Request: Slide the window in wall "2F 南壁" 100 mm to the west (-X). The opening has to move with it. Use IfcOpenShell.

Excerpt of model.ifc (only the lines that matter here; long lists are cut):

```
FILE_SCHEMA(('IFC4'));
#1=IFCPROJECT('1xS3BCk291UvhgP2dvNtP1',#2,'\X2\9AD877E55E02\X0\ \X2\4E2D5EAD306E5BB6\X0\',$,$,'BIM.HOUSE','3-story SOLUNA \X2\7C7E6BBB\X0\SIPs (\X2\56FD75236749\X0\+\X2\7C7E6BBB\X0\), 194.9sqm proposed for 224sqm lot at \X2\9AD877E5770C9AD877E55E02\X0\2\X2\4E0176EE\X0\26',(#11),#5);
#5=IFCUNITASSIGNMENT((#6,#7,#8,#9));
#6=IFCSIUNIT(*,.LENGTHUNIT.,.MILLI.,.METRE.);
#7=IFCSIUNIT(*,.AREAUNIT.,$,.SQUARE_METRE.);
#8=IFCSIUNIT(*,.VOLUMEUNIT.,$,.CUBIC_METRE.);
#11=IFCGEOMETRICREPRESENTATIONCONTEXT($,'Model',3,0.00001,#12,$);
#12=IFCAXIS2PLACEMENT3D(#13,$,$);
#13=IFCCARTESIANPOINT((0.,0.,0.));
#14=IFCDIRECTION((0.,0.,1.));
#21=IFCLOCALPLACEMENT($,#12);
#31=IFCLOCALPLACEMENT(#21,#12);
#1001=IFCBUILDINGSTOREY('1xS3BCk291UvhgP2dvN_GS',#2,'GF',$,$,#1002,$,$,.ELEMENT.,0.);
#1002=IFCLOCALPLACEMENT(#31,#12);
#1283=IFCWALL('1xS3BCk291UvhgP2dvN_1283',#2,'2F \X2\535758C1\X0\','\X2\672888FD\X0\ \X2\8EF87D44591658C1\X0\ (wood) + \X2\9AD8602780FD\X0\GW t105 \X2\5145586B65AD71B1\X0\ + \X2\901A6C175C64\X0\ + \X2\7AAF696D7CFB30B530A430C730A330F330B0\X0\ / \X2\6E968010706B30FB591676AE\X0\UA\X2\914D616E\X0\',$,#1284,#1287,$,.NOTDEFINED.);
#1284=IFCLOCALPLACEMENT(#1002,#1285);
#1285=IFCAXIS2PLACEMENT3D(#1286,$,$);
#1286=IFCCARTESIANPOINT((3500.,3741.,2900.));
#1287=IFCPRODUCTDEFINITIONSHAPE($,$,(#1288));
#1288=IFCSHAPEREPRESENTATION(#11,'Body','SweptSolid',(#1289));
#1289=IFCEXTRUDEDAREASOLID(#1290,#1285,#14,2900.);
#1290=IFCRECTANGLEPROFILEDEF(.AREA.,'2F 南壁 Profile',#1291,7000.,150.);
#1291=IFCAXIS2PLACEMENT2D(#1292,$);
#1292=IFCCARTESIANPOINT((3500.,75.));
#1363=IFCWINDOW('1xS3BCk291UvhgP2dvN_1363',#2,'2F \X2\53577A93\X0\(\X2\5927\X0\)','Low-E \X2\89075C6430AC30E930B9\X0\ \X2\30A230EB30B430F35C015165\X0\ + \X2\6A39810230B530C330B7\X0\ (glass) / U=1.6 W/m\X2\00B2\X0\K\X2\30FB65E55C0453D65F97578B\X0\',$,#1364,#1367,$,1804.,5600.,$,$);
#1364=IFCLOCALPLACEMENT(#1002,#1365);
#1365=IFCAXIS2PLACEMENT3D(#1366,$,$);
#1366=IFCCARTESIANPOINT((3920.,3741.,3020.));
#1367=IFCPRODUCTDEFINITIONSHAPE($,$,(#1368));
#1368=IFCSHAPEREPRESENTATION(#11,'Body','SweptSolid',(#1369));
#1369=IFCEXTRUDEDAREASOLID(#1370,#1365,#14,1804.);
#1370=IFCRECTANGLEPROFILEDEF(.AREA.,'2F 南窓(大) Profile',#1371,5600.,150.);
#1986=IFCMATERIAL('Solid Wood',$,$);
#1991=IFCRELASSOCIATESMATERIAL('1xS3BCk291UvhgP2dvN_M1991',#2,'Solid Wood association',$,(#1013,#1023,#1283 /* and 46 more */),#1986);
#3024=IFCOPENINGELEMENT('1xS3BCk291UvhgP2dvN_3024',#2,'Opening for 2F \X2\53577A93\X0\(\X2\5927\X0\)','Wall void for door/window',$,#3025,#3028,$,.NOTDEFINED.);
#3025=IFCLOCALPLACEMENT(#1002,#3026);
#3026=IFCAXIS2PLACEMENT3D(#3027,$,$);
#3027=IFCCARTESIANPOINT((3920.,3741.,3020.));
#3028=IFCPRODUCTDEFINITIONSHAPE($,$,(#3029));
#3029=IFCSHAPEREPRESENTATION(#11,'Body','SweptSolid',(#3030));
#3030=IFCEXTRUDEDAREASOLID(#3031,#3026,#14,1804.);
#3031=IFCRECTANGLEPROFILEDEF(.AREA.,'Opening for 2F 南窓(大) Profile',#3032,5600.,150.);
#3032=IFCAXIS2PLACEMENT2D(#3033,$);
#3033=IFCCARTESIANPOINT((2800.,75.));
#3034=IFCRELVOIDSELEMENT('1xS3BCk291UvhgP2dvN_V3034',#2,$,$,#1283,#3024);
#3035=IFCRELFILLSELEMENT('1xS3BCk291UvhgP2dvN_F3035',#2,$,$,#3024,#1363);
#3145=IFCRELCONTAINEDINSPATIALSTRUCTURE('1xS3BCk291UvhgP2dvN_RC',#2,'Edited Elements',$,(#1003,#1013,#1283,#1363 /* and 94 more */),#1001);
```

```python
import ifcopenshell
import ifcopenshell.api.geometry
import ifcopenshell.util.placement
import ifcopenshell.util.unit

model = ifcopenshell.open("model.ifc")
unit_scale = ifcopenshell.util.unit.calculate_unit_scale(model)

window = model.by_guid("1xS3BCk291UvhgP2dvN_1363")
opening = window.FillsVoids[0].RelatingOpeningElement
wall = opening.VoidsElements[0].RelatingBuildingElement

wall_matrix = ifcopenshell.util.placement.get_local_placement(wall.ObjectPlacement)
shift = wall_matrix[:3, 0] * -0.1 / unit_scale
before = ifcopenshell.util.placement.get_local_placement(window.ObjectPlacement)[:3, 3].copy()

# The window is not placed relative to its opening, so move both.
for product in (opening, window):
    matrix = ifcopenshell.util.placement.get_local_placement(product.ObjectPlacement)
    matrix[:3, 3] += shift
    ifcopenshell.api.geometry.edit_object_placement(model, product=product, matrix=matrix, is_si=False)

after = ifcopenshell.util.placement.get_local_placement(window.ObjectPlacement)[:3, 3]
print("window moved by", (after - before).round(3) + 0.0)

model.write("model_updated.ifc")
```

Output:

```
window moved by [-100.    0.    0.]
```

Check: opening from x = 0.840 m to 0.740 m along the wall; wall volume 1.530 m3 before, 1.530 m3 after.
